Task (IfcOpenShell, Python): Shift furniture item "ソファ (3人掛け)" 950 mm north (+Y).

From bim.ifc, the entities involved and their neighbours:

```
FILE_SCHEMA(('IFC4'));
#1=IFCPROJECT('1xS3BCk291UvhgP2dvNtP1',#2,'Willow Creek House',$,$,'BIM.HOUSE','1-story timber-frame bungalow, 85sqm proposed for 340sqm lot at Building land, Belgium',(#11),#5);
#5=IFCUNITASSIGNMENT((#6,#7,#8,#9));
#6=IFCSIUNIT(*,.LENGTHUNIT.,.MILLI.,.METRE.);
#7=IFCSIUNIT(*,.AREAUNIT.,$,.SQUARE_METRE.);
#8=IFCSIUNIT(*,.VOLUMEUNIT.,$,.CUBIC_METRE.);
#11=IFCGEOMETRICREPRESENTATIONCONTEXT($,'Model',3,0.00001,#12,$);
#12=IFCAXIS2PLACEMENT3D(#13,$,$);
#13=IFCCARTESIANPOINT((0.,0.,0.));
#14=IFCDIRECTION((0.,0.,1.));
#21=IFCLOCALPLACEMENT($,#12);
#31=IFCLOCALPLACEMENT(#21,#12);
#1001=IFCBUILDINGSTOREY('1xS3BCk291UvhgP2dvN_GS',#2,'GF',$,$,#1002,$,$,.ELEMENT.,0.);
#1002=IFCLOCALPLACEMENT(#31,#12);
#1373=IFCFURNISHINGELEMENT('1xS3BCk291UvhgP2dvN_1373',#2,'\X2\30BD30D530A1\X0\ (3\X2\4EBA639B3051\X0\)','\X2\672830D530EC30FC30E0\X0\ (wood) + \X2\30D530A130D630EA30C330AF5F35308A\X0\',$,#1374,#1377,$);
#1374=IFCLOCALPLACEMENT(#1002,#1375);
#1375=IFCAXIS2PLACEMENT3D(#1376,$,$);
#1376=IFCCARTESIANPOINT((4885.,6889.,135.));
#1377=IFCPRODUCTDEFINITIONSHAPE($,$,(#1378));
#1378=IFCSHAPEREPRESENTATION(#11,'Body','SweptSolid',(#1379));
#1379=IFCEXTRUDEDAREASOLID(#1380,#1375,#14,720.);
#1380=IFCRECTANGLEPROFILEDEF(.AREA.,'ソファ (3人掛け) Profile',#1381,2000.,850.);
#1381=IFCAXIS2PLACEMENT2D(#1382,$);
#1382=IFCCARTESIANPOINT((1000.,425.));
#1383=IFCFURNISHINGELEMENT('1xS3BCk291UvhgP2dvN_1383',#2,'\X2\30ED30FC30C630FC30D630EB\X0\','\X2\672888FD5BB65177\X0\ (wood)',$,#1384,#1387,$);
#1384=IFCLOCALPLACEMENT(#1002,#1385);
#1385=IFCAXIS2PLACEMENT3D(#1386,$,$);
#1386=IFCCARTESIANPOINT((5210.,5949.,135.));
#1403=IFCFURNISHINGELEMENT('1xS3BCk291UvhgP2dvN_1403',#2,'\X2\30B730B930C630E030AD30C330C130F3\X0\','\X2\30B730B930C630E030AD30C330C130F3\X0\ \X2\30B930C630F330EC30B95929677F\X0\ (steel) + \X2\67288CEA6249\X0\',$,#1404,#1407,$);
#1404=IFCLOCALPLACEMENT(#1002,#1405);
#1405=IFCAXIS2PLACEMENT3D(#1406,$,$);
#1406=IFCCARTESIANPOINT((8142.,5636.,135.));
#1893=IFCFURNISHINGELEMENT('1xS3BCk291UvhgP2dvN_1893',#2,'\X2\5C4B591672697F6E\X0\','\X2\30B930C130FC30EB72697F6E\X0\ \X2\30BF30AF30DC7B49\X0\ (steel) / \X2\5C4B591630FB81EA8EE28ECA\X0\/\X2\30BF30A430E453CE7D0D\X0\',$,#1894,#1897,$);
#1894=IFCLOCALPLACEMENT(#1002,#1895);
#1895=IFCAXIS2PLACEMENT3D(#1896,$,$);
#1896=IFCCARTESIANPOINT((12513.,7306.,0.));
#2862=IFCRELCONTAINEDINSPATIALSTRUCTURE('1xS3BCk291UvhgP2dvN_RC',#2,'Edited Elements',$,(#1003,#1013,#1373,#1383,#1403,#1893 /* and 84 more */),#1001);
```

```python
import ifcopenshell
import ifcopenshell.api.geometry
import ifcopenshell.util.placement
import ifcopenshell.util.unit

model = ifcopenshell.open("bim.ifc")
unit_scale = ifcopenshell.util.unit.calculate_unit_scale(model)

item = model.by_guid("1xS3BCk291UvhgP2dvN_1373")
matrix = ifcopenshell.util.placement.get_local_placement(item.ObjectPlacement)
matrix[1, 3] += 0.95 / unit_scale
ifcopenshell.api.geometry.edit_object_placement(model, product=item, matrix=matrix, is_si=False)

print(ifcopenshell.util.placement.get_local_placement(item.ObjectPlacement).round(3) + 0.0)

model.write("bim_rev.ifc")
```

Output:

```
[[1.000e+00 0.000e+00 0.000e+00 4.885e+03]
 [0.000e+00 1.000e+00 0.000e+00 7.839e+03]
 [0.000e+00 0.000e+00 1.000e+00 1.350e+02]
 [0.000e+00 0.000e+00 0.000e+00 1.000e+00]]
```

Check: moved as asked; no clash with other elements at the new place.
